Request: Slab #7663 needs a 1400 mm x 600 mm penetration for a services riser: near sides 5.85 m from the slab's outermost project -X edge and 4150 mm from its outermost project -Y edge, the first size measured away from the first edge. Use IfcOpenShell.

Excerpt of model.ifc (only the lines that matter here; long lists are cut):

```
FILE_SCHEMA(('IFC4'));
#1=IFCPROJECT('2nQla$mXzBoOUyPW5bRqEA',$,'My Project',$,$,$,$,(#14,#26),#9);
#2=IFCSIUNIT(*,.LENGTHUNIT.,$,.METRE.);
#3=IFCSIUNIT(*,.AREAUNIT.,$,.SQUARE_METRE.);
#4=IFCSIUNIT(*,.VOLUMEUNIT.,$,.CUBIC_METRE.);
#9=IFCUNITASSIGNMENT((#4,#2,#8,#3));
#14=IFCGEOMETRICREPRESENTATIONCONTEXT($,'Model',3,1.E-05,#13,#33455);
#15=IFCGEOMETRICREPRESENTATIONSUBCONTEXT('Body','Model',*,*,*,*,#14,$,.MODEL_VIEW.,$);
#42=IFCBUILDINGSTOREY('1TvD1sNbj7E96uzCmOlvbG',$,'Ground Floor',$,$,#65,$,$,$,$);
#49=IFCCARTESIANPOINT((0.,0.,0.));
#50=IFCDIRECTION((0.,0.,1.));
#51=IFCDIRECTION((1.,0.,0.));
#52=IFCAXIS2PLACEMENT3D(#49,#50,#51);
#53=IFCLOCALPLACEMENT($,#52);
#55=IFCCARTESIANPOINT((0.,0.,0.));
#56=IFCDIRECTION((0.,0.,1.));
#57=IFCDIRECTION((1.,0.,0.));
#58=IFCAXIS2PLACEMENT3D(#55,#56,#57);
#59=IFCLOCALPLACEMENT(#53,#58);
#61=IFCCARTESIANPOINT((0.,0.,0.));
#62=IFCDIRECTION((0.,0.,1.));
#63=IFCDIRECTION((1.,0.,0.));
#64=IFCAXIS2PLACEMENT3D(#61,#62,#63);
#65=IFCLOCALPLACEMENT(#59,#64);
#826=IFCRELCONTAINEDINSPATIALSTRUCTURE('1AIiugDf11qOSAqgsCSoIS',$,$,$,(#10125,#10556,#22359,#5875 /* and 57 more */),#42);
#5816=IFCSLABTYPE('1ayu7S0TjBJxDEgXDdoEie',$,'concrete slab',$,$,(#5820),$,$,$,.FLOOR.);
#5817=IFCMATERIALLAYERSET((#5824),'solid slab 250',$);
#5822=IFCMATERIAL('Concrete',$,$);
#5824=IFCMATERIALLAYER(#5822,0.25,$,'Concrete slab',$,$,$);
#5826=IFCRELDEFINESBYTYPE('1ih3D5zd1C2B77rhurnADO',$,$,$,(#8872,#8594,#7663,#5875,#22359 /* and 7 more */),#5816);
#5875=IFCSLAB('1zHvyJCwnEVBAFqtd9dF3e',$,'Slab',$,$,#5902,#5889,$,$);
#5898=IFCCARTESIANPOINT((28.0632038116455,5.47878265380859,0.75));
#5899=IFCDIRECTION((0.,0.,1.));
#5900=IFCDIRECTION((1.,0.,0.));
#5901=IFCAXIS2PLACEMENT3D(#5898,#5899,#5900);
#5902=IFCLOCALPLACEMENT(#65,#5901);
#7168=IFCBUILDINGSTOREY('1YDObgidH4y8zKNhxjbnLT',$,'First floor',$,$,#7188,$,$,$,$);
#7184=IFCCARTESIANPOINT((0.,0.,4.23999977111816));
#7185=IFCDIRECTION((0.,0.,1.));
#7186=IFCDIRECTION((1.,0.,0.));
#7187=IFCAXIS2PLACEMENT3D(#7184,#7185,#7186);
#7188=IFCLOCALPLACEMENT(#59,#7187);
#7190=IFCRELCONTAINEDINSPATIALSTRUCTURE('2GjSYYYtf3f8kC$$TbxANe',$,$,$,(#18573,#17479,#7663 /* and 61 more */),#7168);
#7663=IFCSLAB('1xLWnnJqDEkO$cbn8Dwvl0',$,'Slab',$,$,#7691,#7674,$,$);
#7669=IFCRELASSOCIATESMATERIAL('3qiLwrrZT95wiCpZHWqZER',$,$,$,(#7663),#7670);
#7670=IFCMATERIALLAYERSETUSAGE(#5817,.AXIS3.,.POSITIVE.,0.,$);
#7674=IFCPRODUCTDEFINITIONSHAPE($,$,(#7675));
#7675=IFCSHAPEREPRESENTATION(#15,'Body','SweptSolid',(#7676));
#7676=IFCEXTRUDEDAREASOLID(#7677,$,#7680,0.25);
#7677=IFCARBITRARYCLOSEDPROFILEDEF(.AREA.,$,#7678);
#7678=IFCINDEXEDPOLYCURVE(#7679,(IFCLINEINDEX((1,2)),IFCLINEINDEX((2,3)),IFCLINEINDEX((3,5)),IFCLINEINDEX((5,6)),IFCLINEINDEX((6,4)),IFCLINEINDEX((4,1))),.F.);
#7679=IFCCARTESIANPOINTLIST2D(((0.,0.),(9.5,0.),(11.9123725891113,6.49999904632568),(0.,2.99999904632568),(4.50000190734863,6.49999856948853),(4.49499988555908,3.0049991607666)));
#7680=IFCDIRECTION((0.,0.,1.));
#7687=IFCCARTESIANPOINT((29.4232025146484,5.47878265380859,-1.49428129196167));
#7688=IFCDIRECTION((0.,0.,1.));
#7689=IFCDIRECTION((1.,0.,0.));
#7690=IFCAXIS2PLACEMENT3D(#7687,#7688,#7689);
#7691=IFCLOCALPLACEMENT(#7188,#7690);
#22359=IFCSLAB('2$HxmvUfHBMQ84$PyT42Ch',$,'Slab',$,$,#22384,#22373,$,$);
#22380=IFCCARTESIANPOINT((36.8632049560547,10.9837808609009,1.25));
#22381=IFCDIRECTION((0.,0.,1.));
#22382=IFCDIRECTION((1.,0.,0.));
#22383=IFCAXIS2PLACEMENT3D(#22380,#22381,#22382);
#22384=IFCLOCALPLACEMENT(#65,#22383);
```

```python
import numpy as np
import ifcopenshell
import ifcopenshell.api.feature
import ifcopenshell.api.geometry
import ifcopenshell.api.root
import ifcopenshell.geom
import ifcopenshell.util.placement
import ifcopenshell.util.representation
import ifcopenshell.util.shape
import ifcopenshell.util.unit

model = ifcopenshell.open("model.ifc")
unit_scale = ifcopenshell.util.unit.calculate_unit_scale(model)
settings = ifcopenshell.geom.settings()


def volume(element):
    """Net volume in cubic metres, openings subtracted."""
    shape = ifcopenshell.geom.create_shape(settings, element)
    return ifcopenshell.util.shape.get_volume(shape.geometry)


slab = model.by_guid("1xLWnnJqDEkO$cbn8Dwvl0")
before = volume(slab)

# Extent in the slab's own axes, in metres. The edges named are its -X and -Y sides.
slab_shape = ifcopenshell.geom.create_shape(settings, slab)
vertices = ifcopenshell.util.shape.get_vertices(slab_shape.geometry)
x_min, y_min, bottom = vertices.min(axis=0)
top = vertices[:, 2].max()

opening = ifcopenshell.api.root.create_entity(model, ifc_class="IfcOpeningElement", name="Services riser opening", predefined_type="OPENING")
context = ifcopenshell.util.representation.get_context(model, "Model", "Body", "MODEL_VIEW")
width, depth = 1.4, 0.6
outline = [(0.0, 0.0), (width, 0.0), (width, depth), (0.0, depth), (0.0, 0.0)]
# Overshoot both faces by 50 mm so the cut is clean.
shape = ifcopenshell.api.geometry.add_slab_representation(
    model, context=context, depth=top - bottom + 0.1, polyline=outline
)
ifcopenshell.api.geometry.assign_representation(model, product=opening, representation=shape)

matrix = ifcopenshell.util.placement.get_local_placement(slab.ObjectPlacement)
matrix[:, 3] = matrix @ np.append(np.array([x_min + 5.85, y_min + 4.15, bottom - 0.05]) / unit_scale, 1.0)
ifcopenshell.api.geometry.edit_object_placement(model, product=opening, matrix=matrix, is_si=False)
ifcopenshell.api.feature.add_feature(model, feature=opening, element=slab)

after = volume(slab)

print(f"slab volume {before:.3f} -> {after:.3f} m3")

model.write("model_edited.ifc")
```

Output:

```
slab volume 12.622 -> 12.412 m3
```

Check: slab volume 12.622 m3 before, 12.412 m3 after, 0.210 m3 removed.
